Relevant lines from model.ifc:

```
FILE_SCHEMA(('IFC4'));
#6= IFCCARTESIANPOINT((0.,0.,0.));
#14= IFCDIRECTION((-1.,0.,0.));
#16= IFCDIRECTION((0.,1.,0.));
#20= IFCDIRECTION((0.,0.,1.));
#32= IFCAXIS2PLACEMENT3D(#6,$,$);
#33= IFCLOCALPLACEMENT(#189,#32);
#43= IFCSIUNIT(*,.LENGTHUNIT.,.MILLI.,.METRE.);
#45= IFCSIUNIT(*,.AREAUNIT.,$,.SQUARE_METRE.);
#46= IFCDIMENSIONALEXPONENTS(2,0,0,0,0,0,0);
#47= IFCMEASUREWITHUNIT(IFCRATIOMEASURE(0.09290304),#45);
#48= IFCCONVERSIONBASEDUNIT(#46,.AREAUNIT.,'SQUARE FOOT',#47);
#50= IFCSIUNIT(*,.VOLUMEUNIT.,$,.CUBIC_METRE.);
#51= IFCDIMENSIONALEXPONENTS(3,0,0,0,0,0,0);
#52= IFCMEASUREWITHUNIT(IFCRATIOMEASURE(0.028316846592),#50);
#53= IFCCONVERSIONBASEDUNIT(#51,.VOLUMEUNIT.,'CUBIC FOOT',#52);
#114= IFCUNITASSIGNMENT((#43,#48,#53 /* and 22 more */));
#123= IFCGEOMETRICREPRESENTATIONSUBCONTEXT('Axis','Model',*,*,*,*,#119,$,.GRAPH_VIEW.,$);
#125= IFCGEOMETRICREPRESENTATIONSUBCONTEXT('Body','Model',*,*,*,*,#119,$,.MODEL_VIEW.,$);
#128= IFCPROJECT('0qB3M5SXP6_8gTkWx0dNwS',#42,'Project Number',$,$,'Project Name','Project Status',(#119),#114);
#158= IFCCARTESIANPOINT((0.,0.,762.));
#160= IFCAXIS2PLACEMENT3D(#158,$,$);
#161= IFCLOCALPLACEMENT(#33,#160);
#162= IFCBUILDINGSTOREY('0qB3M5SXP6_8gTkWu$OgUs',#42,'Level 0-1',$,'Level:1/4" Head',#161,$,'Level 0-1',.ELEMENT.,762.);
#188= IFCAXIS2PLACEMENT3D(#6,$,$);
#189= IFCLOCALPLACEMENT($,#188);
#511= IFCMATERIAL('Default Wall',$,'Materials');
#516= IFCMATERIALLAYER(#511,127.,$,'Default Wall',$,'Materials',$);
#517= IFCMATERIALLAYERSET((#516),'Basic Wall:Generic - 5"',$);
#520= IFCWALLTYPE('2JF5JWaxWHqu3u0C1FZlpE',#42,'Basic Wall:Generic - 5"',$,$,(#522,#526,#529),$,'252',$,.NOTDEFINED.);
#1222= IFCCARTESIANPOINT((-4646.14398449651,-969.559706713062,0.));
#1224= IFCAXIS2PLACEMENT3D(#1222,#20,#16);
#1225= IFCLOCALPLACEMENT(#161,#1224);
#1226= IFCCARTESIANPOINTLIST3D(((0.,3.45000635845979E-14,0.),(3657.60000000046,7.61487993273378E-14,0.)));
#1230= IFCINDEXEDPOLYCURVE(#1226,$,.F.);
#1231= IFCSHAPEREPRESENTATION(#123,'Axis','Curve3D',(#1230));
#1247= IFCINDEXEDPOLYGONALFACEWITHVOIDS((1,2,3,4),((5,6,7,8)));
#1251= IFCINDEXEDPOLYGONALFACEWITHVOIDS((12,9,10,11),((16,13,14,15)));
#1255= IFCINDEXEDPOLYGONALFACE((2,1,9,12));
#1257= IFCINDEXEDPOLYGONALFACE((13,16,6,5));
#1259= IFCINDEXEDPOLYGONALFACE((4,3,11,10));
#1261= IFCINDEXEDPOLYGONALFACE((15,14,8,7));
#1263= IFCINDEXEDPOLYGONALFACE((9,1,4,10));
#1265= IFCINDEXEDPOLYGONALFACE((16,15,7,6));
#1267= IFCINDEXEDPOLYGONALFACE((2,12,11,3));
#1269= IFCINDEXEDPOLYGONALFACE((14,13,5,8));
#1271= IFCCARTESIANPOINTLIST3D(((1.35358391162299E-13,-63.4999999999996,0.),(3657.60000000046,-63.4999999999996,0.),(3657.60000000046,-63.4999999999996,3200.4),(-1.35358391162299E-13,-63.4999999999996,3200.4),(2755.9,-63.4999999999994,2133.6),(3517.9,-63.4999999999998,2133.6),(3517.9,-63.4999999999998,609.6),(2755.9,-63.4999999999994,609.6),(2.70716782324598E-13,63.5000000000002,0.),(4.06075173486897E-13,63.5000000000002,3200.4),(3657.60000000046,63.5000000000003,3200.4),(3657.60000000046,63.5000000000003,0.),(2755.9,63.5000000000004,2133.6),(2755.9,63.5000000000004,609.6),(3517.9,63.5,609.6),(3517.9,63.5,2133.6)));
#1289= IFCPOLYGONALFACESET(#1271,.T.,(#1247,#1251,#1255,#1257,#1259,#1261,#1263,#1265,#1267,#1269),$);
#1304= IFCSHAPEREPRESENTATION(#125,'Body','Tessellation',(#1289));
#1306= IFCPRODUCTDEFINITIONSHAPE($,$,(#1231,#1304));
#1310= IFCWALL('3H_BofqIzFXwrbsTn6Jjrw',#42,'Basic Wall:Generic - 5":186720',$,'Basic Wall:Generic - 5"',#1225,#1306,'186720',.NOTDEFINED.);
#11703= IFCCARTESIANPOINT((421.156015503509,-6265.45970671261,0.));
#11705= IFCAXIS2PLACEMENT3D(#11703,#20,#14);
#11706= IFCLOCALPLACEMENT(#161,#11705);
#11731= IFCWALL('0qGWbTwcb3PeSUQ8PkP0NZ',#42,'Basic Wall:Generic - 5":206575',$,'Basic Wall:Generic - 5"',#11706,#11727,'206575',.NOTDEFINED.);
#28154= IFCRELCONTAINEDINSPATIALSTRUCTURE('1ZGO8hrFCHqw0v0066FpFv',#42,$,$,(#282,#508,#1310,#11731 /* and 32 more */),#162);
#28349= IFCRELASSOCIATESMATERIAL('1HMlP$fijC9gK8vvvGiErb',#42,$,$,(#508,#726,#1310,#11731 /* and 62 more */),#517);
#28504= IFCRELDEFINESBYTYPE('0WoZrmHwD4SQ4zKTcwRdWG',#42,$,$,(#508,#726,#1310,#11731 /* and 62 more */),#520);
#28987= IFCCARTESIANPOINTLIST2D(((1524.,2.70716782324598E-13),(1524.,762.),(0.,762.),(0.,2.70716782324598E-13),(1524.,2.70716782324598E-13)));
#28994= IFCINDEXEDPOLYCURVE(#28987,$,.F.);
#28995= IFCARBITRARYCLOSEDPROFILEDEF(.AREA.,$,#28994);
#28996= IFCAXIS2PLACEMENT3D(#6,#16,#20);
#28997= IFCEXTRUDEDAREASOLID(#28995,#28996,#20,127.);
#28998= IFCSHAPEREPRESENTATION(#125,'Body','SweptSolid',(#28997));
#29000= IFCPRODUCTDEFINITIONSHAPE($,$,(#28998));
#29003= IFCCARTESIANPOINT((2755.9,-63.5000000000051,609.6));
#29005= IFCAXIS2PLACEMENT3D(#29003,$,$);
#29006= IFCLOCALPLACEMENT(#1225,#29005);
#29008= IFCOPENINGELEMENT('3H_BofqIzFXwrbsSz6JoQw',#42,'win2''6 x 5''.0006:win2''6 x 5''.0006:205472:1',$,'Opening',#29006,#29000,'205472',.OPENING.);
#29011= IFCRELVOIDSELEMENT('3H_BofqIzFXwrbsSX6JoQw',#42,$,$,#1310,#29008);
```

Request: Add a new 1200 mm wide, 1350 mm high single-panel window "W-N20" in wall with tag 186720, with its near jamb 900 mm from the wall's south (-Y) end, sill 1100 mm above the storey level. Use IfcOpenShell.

```python
import numpy as np
import ifcopenshell
import ifcopenshell.api.feature
import ifcopenshell.api.geometry
import ifcopenshell.api.root
import ifcopenshell.api.spatial
import ifcopenshell.geom
import ifcopenshell.util.element
import ifcopenshell.util.placement
import ifcopenshell.util.representation
import ifcopenshell.util.shape
import ifcopenshell.util.unit

model = ifcopenshell.open("model.ifc")
unit_scale = ifcopenshell.util.unit.calculate_unit_scale(model)
settings = ifcopenshell.geom.settings()


def volume(element):
    """Net volume in cubic metres, openings subtracted."""
    shape = ifcopenshell.geom.create_shape(settings, element)
    return ifcopenshell.util.shape.get_volume(shape.geometry)


wall = model.by_guid("3H_BofqIzFXwrbsTn6Jjrw")
storey = ifcopenshell.util.element.get_container(wall, ifc_class="IfcBuildingStorey")
context = ifcopenshell.util.representation.get_context(model, "Model", "Body", "MODEL_VIEW")
before = volume(wall)

width, height, from_end, sill = 1.2, 1.35, 0.9, 1.1  # metres

# The wall runs along its own X axis, and the end named is its -X end.
wall_shape = ifcopenshell.geom.create_shape(settings, wall)
x, y, z = ifcopenshell.util.shape.get_vertices(wall_shape.geometry).T
start = x.min() + from_end
face, thickness = float(y.min()), float(y.max() - y.min())
wall_matrix = ifcopenshell.util.placement.get_local_placement(wall.ObjectPlacement)
level = ifcopenshell.util.placement.get_local_placement(storey.ObjectPlacement)[2, 3]


def in_wall(x, y):
    """Placement at x, y metres in the wall's axes, at sill height."""
    matrix = wall_matrix.copy()
    matrix[:, 3] = wall_matrix @ np.array([x / unit_scale, y / unit_scale, 0.0, 1.0])
    matrix[2, 3] = level + sill / unit_scale
    return matrix


# Opening: a box that overshoots both wall faces by 50 mm.
opening = ifcopenshell.api.root.create_entity(model, ifc_class="IfcOpeningElement", predefined_type="OPENING")
box = ifcopenshell.api.geometry.add_wall_representation(
    model, context=context, length=width, height=height, thickness=thickness + 0.1
)
ifcopenshell.api.geometry.assign_representation(model, product=opening, representation=box)
ifcopenshell.api.geometry.edit_object_placement(model, product=opening, matrix=in_wall(start, face - 0.05), is_si=False)
ifcopenshell.api.feature.add_feature(model, feature=opening, element=wall)

window = ifcopenshell.api.root.create_entity(model, ifc_class="IfcWindow", name="W-N20", predefined_type="WINDOW")
window.OverallWidth, window.OverallHeight = width / unit_scale, height / unit_scale
window.PartitioningType = "SINGLE_PANEL"
body = ifcopenshell.api.geometry.add_window_representation(
    model,
    context=context,
    overall_width=window.OverallWidth,
    overall_height=window.OverallHeight,
    partition_type="SINGLE_PANEL",
)
ifcopenshell.api.geometry.assign_representation(model, product=window, representation=body)
ifcopenshell.api.spatial.assign_container(model, products=[window], relating_structure=storey)
ifcopenshell.api.feature.add_filling(model, opening=opening, element=window)

# Centre the window in the wall's thickness.
ifcopenshell.api.geometry.edit_object_placement(model, product=window, matrix=in_wall(start, face), is_si=False)
window_shape = ifcopenshell.geom.create_shape(settings, window)
depth = ifcopenshell.util.shape.get_vertices(window_shape.geometry)[:, 1]
offset = face + thickness / 2 - (depth.min() + depth.max()) / 2
ifcopenshell.api.geometry.edit_object_placement(model, product=window, matrix=in_wall(start, offset), is_si=False)

after = volume(wall)

print(f"wall volume {before:.3f} -> {after:.3f} m3")

model.write("model-out.ifc")
```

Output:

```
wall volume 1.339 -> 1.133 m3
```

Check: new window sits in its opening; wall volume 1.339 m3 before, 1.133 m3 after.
